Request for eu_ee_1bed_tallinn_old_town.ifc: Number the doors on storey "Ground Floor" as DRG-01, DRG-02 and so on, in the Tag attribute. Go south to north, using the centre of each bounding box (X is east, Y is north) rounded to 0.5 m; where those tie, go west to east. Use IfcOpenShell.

First a look at what the model holds.

```python
import ifcopenshell
import ifcopenshell.util.element
import ifcopenshell.util.placement

model = ifcopenshell.open("eu_ee_1bed_tallinn_old_town.ifc")
print(model.schema)
storey = next(s for s in model.by_type("IfcBuildingStorey") if s.Name == "Ground Floor")
doors = [e for e in ifcopenshell.util.element.get_decomposition(storey) if e.is_a("IfcDoor")]
for e in sorted(doors, key=lambda e: e.id()):
    origin = ifcopenshell.util.placement.get_local_placement(e.ObjectPlacement)[:3, 3]
    print(e.id(), e.Tag, e.Name, origin.round(2) + 0.0, sep=" | ")
```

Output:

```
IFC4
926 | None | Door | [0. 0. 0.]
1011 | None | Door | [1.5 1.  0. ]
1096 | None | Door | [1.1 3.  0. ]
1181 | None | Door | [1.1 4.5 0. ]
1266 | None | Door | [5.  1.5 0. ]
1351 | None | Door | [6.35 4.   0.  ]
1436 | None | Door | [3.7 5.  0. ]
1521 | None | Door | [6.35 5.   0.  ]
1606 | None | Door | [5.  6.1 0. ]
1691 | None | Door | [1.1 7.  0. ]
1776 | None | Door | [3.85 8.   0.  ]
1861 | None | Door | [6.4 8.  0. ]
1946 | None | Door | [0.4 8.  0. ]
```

```python
import ifcopenshell
import ifcopenshell.geom
import ifcopenshell.util.element
import ifcopenshell.util.shape

model = ifcopenshell.open("eu_ee_1bed_tallinn_old_town.ifc")
settings = ifcopenshell.geom.settings()
settings.set("use-world-coords", True)


def centre(element):
    shape = ifcopenshell.geom.create_shape(settings, element)
    return ifcopenshell.util.shape.get_bbox_centroid(shape.geometry)


storey = next(s for s in model.by_type("IfcBuildingStorey") if s.Name == "Ground Floor")
doors = [e for e in ifcopenshell.util.element.get_decomposition(storey) if e.is_a("IfcDoor")]

# Insertion points can sit at a corner or the storey origin, so sort by the geometry (in metres).
centres = {e: centre(e) for e in doors}
doors.sort(key=lambda e: (round(centres[e][1] / 0.5), centres[e][0]))

for i, e in enumerate(doors, start=1):
    number = f"DRG-{i:02d}"
    e.Tag = number
    print(e.id(), number)

model.write("eu_ee_1bed_tallinn_old_town_edited.ifc")
```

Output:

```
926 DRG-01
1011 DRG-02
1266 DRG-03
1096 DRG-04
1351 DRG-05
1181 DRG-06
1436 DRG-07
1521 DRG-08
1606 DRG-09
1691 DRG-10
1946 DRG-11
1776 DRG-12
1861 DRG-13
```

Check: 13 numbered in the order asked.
